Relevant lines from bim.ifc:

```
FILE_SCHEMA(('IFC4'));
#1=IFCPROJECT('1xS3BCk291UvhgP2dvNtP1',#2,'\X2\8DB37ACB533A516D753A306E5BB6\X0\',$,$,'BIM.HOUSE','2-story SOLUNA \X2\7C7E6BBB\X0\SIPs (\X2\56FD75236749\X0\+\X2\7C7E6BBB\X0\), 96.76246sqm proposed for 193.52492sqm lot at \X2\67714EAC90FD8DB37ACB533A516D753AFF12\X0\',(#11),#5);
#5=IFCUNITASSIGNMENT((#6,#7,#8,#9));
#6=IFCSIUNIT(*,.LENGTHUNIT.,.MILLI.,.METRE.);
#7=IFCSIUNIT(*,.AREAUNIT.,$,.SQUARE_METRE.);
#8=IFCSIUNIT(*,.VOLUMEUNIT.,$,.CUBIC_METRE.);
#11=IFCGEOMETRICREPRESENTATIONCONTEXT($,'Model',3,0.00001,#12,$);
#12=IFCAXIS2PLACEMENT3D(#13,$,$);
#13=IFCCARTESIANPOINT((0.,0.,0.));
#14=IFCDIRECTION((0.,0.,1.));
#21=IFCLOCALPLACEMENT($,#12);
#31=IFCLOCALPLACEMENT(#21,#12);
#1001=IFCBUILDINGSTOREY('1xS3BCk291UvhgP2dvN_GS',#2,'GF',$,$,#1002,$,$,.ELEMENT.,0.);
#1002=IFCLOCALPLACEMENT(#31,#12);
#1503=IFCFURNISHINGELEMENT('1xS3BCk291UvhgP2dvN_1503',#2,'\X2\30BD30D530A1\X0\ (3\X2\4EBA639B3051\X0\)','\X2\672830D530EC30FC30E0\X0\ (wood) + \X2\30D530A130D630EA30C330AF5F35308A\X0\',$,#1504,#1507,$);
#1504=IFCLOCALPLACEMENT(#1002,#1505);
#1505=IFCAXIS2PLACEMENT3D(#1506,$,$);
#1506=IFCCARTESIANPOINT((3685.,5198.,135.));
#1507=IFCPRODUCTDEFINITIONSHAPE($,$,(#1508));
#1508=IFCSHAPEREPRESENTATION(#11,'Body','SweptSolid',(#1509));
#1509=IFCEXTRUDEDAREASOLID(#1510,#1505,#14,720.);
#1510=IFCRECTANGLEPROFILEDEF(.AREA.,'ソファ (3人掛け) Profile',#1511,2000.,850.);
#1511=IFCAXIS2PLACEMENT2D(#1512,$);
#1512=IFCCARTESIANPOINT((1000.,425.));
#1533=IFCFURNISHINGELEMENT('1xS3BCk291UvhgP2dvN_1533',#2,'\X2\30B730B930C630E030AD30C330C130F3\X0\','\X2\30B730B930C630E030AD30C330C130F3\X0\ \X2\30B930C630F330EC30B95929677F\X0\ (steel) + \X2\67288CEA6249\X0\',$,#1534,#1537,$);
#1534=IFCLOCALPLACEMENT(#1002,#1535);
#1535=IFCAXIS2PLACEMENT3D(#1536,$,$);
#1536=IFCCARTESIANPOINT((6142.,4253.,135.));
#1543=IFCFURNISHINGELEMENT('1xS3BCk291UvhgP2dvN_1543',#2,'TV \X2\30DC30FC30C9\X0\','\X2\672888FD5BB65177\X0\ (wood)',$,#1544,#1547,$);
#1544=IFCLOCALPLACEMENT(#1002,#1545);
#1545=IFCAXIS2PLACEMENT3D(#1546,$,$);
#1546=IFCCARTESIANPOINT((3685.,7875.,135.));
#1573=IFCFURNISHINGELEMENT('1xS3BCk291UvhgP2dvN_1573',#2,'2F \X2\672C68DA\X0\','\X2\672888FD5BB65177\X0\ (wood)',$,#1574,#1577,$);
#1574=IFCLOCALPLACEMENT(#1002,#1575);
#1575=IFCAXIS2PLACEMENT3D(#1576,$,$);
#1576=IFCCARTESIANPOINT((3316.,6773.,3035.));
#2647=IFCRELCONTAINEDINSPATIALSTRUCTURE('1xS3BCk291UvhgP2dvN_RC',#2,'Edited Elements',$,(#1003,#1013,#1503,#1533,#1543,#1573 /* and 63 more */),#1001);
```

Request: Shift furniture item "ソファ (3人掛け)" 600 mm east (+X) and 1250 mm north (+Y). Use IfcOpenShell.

```python
import ifcopenshell
import ifcopenshell.api.geometry
import ifcopenshell.util.placement
import ifcopenshell.util.unit

model = ifcopenshell.open("bim.ifc")
unit_scale = ifcopenshell.util.unit.calculate_unit_scale(model)

item = model.by_id(1503)
matrix = ifcopenshell.util.placement.get_local_placement(item.ObjectPlacement)
matrix[0, 3] += 0.6 / unit_scale
matrix[1, 3] += 1.25 / unit_scale
ifcopenshell.api.geometry.edit_object_placement(model, product=item, matrix=matrix, is_si=False)

print(ifcopenshell.util.placement.get_local_placement(item.ObjectPlacement).round(3) + 0.0)

model.write("bim_updated.ifc")
```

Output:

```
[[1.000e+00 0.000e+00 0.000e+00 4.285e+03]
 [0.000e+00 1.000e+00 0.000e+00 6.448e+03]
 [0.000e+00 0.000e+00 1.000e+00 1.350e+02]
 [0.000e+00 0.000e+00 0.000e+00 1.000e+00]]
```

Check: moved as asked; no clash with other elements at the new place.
